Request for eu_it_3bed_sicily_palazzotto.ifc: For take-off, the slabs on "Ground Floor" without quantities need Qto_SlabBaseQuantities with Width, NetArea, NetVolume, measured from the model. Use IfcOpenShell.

First a look at what the model holds.

```python
import ifcopenshell
import ifcopenshell.util.element
import ifcopenshell.util.unit

model = ifcopenshell.open("eu_it_3bed_sicily_palazzotto.ifc")
print(model.schema)
for unit_type in ("LENGTHUNIT", "AREAUNIT", "VOLUMEUNIT"):
    print(unit_type, ifcopenshell.util.unit.calculate_unit_scale(model, unit_type))
storey = next(s for s in model.by_type("IfcBuildingStorey") if s.Name == "Ground Floor")
slabs = [e for e in ifcopenshell.util.element.get_decomposition(storey) if e.is_a("IfcSlab")]
for e in sorted(slabs, key=lambda e: e.id()):
    print(e.id(), e.is_a(), e.Name, list(ifcopenshell.util.element.get_psets(e, qtos_only=True)), sep=" | ")
```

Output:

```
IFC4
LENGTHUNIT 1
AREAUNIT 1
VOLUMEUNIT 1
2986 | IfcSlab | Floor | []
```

```python
import ifcopenshell
import ifcopenshell.api.pset
import ifcopenshell.geom
import ifcopenshell.util.element
import ifcopenshell.util.shape
import ifcopenshell.util.unit

model = ifcopenshell.open("eu_it_3bed_sicily_palazzotto.ifc")
unit_scale = ifcopenshell.util.unit.calculate_unit_scale(model)
area_scale = ifcopenshell.util.unit.calculate_unit_scale(model, "AREAUNIT")
volume_scale = ifcopenshell.util.unit.calculate_unit_scale(model, "VOLUMEUNIT")
settings = ifcopenshell.geom.settings()

storey = next(s for s in model.by_type("IfcBuildingStorey") if s.Name == "Ground Floor")
slabs = [e for e in ifcopenshell.util.element.get_decomposition(storey) if e.is_a("IfcSlab")]

for e in sorted(slabs, key=lambda e: e.id()):
    if ifcopenshell.util.element.get_psets(e, qtos_only=True, should_inherit=False):
        continue
    # Geometry comes back in metres, in the element's own axes.
    shape = ifcopenshell.geom.create_shape(settings, e)
    values = {
        "Width": ifcopenshell.util.shape.get_z(shape.geometry) / unit_scale,
        "NetArea": ifcopenshell.util.shape.get_footprint_area(shape.geometry) / area_scale,
        "NetVolume": ifcopenshell.util.shape.get_volume(shape.geometry) / volume_scale,
    }
    qto = ifcopenshell.api.pset.add_qto(model, product=e, name="Qto_SlabBaseQuantities")
    ifcopenshell.api.pset.edit_qto(model, qto=qto, properties=values)
    print(e.id(), {k: round(v, 3) for k, v in values.items()})

model.write("eu_it_3bed_sicily_palazzotto_rev.ifc")
```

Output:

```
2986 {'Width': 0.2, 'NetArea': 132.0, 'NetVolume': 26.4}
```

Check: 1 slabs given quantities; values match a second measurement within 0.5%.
